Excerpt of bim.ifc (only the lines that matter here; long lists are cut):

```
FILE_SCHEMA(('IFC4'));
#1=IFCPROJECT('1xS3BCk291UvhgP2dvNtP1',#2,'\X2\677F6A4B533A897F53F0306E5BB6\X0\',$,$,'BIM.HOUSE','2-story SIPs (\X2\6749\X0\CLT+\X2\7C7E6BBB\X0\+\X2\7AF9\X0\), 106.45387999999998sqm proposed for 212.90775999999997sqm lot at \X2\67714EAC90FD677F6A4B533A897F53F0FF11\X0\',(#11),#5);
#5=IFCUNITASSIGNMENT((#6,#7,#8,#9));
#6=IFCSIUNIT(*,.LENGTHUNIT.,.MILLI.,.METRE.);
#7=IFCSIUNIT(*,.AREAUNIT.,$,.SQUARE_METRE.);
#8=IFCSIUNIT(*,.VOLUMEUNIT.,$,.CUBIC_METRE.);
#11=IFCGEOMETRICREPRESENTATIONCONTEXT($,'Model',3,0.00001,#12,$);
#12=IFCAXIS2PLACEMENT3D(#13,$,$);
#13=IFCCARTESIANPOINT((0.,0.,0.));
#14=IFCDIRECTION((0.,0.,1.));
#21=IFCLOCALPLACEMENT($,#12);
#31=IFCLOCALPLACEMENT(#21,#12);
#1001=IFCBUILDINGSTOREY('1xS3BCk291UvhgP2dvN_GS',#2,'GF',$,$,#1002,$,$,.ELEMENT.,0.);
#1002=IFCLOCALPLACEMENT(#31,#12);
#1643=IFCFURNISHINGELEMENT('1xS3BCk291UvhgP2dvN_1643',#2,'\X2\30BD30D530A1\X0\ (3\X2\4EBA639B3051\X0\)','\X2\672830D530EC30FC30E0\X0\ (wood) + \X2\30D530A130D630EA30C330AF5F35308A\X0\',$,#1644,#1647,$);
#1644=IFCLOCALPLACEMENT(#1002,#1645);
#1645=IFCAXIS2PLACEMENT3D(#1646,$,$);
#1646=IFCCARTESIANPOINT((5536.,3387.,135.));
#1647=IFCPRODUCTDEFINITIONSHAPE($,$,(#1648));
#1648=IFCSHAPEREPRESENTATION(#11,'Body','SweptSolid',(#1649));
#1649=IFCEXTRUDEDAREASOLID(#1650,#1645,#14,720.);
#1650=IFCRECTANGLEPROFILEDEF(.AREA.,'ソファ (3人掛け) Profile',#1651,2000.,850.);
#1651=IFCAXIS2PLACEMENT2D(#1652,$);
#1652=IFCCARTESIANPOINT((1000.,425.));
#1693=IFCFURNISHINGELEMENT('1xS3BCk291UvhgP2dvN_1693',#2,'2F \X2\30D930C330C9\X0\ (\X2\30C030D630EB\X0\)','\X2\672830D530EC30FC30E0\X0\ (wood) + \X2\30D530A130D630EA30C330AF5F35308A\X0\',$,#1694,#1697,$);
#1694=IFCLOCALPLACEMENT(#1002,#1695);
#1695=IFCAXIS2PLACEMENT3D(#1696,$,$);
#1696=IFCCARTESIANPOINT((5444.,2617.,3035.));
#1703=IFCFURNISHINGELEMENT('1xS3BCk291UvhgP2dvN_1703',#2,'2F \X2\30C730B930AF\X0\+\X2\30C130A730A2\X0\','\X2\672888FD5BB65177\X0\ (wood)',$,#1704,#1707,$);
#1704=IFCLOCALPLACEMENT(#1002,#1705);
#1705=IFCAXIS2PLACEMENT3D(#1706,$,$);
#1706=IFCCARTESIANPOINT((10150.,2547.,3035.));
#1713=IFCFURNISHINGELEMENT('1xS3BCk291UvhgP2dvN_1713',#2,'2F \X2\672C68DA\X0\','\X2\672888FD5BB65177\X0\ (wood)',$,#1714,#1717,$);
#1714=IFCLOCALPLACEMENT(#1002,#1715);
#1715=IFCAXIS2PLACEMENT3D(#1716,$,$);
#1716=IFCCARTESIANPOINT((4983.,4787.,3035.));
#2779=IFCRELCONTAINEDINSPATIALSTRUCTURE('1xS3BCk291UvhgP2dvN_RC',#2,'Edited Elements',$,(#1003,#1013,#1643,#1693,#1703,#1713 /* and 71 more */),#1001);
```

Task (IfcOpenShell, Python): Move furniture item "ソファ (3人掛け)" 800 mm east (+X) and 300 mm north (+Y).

```python
import ifcopenshell
import ifcopenshell.api.geometry
import ifcopenshell.util.placement

model = ifcopenshell.open("bim.ifc")

item = model.by_id(1643)
matrix = ifcopenshell.util.placement.get_local_placement(item.ObjectPlacement)
matrix[0, 3] += 800.0
matrix[1, 3] += 300.0
ifcopenshell.api.geometry.edit_object_placement(model, product=item, matrix=matrix, is_si=False)

print(ifcopenshell.util.placement.get_local_placement(item.ObjectPlacement).round(3) + 0.0)

model.write("bim_rev.ifc")
```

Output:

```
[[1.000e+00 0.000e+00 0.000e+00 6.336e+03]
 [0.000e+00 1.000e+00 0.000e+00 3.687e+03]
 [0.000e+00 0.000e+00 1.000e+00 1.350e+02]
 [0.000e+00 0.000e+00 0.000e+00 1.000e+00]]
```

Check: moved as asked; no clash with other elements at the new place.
